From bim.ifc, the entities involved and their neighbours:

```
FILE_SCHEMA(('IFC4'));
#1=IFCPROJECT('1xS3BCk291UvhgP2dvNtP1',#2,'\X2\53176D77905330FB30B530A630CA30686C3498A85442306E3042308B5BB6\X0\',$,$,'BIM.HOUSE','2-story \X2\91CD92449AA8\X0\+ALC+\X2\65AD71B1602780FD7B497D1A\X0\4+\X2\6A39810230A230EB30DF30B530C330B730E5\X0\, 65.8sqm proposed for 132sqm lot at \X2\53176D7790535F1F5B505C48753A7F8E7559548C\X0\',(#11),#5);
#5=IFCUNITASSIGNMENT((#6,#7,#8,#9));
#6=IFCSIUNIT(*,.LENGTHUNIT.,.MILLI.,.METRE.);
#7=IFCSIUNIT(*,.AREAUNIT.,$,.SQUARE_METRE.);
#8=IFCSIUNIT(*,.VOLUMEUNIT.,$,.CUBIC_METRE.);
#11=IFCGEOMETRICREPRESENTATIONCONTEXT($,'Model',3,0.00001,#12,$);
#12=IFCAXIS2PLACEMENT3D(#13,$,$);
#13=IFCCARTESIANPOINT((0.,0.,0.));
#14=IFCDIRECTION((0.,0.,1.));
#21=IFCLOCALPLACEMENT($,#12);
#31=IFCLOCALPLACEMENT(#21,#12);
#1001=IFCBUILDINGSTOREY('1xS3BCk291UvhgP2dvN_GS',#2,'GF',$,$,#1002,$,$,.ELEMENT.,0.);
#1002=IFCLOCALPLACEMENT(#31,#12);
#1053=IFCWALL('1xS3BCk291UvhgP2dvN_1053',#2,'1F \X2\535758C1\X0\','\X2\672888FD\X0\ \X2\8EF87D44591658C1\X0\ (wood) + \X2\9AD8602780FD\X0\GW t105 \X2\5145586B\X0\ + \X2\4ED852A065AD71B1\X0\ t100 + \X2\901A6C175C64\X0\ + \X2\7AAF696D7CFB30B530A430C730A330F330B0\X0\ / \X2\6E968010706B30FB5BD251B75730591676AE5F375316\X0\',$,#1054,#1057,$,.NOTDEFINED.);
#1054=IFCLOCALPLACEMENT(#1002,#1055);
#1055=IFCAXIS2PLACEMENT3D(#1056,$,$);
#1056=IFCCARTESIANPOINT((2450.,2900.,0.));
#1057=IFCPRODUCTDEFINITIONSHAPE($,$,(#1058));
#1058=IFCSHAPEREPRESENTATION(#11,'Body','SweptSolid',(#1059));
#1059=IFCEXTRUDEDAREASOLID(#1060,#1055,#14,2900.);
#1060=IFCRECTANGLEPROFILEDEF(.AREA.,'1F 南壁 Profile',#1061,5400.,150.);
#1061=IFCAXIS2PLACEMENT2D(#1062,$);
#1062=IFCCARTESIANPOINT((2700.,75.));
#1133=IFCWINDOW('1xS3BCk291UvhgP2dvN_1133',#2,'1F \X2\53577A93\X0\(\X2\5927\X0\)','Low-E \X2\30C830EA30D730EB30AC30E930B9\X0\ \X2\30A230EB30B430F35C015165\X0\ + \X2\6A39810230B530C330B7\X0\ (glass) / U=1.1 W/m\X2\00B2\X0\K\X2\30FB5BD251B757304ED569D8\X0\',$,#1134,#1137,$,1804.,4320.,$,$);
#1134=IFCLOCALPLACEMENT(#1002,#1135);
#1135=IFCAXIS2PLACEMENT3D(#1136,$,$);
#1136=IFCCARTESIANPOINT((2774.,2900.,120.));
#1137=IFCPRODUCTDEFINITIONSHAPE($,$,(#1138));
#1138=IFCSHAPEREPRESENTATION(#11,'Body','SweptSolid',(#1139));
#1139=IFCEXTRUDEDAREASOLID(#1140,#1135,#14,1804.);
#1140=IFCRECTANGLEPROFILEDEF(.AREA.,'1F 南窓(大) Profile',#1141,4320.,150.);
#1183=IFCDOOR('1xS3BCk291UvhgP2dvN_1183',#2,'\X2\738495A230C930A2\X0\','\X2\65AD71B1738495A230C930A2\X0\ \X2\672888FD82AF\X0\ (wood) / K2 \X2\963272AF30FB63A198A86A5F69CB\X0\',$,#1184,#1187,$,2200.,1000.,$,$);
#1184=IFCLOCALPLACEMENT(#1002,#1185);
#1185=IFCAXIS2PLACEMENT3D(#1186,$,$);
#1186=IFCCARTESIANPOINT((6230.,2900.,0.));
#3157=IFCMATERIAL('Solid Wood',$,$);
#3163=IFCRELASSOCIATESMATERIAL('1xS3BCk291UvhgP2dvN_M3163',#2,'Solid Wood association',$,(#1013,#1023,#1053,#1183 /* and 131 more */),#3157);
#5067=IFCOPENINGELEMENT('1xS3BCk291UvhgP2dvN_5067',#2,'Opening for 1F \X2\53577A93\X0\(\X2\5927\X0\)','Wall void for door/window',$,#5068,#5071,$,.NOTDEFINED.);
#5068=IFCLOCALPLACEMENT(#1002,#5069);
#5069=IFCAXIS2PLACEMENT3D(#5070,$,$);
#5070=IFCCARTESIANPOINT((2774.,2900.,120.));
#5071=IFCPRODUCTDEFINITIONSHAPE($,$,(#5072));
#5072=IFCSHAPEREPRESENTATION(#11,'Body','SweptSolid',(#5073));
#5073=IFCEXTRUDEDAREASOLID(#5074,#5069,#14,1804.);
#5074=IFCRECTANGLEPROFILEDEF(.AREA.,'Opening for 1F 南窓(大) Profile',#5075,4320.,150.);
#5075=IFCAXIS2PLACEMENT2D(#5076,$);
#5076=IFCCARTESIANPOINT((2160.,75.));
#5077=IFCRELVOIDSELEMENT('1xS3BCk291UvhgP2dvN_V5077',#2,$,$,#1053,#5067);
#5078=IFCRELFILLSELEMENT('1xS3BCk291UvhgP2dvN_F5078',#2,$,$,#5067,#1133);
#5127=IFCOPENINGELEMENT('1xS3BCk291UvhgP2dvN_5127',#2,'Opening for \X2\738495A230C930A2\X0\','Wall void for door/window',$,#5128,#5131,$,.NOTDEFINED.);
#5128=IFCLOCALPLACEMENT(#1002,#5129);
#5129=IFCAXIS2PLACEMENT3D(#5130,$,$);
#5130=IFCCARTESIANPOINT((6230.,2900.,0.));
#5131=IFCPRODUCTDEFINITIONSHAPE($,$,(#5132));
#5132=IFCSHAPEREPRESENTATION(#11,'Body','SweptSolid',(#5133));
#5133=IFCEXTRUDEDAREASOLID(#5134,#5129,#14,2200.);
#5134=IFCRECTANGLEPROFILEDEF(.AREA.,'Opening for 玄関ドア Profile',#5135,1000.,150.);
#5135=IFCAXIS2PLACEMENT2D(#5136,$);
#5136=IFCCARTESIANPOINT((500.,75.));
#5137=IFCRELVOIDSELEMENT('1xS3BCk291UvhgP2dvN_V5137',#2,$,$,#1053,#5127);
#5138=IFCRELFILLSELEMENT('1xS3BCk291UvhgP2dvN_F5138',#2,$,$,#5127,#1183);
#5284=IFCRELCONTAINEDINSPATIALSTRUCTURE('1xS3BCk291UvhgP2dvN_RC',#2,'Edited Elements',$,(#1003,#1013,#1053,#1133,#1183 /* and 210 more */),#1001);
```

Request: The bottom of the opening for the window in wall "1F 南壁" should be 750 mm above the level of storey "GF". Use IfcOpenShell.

```python
import numpy as np
import ifcopenshell
import ifcopenshell.api.geometry
import ifcopenshell.geom
import ifcopenshell.util.element
import ifcopenshell.util.placement
import ifcopenshell.util.shape
import ifcopenshell.util.unit

model = ifcopenshell.open("bim.ifc")
unit_scale = ifcopenshell.util.unit.calculate_unit_scale(model)

window = model.by_guid("1xS3BCk291UvhgP2dvN_1133")
opening = window.FillsVoids[0].RelatingOpeningElement
storey = ifcopenshell.util.element.get_container(window, ifc_class="IfcBuildingStorey")
level = ifcopenshell.util.placement.get_local_placement(storey.ObjectPlacement)[2, 3]

# The opening's origin need not be at the sill, so measure its lowest point.
shape = ifcopenshell.geom.create_shape(ifcopenshell.geom.settings(), opening)
bottom = ifcopenshell.util.shape.get_shape_bottom_elevation(shape, shape.geometry) / unit_scale
dz = level + 0.75 / unit_scale - bottom

shift = np.array([0.0, 0.0, dz])
# The window is not placed relative to its opening, so move both.
for product in (opening, window):
    matrix = ifcopenshell.util.placement.get_local_placement(product.ObjectPlacement)
    matrix[:3, 3] += shift
    ifcopenshell.api.geometry.edit_object_placement(model, product=product, matrix=matrix, is_si=False)

print(f"moved by {dz * unit_scale:+.3f} m")

model.write("bim_updated.ifc")
```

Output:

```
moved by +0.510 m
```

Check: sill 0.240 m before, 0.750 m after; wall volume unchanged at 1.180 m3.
